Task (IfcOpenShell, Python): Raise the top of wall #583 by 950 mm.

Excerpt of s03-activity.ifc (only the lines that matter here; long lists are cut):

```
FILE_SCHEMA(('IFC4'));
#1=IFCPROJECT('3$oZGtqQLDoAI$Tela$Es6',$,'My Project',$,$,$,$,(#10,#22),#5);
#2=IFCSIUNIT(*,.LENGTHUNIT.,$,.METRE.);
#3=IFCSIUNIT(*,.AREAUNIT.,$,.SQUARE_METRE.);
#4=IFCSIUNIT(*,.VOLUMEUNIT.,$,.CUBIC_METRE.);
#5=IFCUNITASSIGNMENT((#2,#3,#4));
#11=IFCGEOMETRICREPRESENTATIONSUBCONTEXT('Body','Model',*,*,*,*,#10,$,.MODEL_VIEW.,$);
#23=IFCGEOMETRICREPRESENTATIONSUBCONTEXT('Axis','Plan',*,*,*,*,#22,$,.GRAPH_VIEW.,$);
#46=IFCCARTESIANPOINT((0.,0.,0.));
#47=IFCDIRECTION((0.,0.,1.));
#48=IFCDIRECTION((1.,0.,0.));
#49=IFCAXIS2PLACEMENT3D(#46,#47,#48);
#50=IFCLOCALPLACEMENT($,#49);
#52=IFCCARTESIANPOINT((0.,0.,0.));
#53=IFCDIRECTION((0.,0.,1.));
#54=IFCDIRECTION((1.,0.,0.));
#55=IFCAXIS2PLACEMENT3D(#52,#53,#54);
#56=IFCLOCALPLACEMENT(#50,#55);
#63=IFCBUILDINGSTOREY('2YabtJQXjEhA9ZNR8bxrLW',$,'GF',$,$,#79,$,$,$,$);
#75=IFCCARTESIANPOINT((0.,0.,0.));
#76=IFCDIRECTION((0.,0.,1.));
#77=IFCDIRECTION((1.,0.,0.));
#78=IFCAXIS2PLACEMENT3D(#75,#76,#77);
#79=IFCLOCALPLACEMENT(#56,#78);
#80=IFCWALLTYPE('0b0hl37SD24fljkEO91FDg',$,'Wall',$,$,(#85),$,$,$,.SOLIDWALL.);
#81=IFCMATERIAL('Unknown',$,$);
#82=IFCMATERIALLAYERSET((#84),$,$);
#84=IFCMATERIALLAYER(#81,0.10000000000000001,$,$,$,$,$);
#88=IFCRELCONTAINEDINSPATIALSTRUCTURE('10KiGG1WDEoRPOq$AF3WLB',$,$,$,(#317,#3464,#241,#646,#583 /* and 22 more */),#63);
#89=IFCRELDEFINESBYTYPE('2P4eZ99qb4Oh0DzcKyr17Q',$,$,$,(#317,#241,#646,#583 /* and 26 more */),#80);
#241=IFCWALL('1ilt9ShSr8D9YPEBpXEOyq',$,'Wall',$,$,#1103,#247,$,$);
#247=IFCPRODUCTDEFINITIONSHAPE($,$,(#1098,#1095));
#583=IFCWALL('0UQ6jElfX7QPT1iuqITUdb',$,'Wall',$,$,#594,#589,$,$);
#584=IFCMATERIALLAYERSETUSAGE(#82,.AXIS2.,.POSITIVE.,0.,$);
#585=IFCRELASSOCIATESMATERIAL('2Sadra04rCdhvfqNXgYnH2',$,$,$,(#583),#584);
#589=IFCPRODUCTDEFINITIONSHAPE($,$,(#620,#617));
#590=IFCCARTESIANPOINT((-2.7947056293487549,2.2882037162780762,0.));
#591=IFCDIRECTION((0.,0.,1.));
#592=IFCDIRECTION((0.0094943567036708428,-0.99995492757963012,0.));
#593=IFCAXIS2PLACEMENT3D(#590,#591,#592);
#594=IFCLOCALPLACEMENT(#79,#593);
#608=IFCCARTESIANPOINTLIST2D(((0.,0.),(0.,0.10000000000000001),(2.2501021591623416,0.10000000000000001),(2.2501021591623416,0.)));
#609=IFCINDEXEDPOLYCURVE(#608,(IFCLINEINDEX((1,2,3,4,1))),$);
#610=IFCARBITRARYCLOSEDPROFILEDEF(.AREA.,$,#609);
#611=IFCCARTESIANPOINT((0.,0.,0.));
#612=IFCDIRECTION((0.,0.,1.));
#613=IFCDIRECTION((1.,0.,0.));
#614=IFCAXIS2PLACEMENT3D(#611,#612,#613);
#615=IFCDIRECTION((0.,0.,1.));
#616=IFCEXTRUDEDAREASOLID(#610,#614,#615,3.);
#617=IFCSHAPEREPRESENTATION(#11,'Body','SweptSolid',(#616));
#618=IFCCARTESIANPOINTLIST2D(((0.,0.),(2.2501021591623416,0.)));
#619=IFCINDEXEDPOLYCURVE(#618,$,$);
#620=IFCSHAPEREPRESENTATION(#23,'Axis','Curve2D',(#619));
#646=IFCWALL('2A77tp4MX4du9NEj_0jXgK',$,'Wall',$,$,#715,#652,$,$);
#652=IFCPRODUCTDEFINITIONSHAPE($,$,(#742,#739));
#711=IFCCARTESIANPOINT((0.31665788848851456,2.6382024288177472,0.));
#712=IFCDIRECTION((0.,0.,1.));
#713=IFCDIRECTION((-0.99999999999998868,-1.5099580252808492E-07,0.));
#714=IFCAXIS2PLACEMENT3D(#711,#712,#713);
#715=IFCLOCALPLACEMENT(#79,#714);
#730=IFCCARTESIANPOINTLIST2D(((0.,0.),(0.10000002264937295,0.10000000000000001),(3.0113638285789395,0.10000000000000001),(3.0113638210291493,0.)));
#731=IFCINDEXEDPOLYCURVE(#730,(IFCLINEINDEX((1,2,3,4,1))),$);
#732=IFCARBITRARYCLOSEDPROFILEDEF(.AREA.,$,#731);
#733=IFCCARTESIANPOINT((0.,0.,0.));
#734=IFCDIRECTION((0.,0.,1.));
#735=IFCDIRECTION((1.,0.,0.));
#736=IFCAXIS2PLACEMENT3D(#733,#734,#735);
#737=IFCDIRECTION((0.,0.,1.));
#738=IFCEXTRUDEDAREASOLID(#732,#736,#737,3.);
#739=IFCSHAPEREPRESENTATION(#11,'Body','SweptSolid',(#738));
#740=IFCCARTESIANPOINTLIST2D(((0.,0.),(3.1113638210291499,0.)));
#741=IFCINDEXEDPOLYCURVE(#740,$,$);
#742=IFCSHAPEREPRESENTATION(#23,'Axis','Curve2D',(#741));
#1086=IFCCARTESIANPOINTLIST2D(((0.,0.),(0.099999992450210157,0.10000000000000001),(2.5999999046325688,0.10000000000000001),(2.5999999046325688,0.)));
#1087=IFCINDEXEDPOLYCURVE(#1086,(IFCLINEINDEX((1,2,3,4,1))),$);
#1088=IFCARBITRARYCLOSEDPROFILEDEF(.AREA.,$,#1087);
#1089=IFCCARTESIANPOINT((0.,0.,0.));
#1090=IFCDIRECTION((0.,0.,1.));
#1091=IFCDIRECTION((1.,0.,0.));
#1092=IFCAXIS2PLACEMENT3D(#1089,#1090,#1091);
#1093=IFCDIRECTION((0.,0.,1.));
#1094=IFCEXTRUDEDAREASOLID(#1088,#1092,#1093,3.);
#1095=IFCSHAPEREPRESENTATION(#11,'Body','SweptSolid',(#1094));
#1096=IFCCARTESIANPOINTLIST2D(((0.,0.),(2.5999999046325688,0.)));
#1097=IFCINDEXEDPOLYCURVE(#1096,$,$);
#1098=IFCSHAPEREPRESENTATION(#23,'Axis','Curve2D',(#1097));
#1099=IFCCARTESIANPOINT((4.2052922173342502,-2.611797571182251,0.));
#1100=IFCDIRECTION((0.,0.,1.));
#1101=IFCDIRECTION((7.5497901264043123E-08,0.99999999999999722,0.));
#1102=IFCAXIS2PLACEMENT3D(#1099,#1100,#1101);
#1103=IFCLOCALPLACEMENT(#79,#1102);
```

```python
import ifcopenshell
import ifcopenshell.geom
import ifcopenshell.util.representation
import ifcopenshell.util.shape
import ifcopenshell.util.unit

model = ifcopenshell.open("s03-activity.ifc")
unit_scale = ifcopenshell.util.unit.calculate_unit_scale(model)
settings = ifcopenshell.geom.settings()


def volume(element):
    """Net volume in cubic metres, openings subtracted."""
    shape = ifcopenshell.geom.create_shape(settings, element)
    return ifcopenshell.util.shape.get_volume(shape.geometry)


wall = model.by_guid("0UQ6jElfX7QPT1iuqITUdb")
before = volume(wall)

body = ifcopenshell.util.representation.get_representation(wall, "Model", "Body")
solid = body.Items[0]
old_height = solid.Depth
solid.Depth += 0.95 / unit_scale
after = volume(wall)

print(f"height {old_height:g} -> {solid.Depth:g}, volume {before:.3f} -> {after:.3f} m3")

model.write("s03-activity_rev.ifc")
```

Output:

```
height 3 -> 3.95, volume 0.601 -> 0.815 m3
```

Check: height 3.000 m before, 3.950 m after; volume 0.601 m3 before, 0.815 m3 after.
